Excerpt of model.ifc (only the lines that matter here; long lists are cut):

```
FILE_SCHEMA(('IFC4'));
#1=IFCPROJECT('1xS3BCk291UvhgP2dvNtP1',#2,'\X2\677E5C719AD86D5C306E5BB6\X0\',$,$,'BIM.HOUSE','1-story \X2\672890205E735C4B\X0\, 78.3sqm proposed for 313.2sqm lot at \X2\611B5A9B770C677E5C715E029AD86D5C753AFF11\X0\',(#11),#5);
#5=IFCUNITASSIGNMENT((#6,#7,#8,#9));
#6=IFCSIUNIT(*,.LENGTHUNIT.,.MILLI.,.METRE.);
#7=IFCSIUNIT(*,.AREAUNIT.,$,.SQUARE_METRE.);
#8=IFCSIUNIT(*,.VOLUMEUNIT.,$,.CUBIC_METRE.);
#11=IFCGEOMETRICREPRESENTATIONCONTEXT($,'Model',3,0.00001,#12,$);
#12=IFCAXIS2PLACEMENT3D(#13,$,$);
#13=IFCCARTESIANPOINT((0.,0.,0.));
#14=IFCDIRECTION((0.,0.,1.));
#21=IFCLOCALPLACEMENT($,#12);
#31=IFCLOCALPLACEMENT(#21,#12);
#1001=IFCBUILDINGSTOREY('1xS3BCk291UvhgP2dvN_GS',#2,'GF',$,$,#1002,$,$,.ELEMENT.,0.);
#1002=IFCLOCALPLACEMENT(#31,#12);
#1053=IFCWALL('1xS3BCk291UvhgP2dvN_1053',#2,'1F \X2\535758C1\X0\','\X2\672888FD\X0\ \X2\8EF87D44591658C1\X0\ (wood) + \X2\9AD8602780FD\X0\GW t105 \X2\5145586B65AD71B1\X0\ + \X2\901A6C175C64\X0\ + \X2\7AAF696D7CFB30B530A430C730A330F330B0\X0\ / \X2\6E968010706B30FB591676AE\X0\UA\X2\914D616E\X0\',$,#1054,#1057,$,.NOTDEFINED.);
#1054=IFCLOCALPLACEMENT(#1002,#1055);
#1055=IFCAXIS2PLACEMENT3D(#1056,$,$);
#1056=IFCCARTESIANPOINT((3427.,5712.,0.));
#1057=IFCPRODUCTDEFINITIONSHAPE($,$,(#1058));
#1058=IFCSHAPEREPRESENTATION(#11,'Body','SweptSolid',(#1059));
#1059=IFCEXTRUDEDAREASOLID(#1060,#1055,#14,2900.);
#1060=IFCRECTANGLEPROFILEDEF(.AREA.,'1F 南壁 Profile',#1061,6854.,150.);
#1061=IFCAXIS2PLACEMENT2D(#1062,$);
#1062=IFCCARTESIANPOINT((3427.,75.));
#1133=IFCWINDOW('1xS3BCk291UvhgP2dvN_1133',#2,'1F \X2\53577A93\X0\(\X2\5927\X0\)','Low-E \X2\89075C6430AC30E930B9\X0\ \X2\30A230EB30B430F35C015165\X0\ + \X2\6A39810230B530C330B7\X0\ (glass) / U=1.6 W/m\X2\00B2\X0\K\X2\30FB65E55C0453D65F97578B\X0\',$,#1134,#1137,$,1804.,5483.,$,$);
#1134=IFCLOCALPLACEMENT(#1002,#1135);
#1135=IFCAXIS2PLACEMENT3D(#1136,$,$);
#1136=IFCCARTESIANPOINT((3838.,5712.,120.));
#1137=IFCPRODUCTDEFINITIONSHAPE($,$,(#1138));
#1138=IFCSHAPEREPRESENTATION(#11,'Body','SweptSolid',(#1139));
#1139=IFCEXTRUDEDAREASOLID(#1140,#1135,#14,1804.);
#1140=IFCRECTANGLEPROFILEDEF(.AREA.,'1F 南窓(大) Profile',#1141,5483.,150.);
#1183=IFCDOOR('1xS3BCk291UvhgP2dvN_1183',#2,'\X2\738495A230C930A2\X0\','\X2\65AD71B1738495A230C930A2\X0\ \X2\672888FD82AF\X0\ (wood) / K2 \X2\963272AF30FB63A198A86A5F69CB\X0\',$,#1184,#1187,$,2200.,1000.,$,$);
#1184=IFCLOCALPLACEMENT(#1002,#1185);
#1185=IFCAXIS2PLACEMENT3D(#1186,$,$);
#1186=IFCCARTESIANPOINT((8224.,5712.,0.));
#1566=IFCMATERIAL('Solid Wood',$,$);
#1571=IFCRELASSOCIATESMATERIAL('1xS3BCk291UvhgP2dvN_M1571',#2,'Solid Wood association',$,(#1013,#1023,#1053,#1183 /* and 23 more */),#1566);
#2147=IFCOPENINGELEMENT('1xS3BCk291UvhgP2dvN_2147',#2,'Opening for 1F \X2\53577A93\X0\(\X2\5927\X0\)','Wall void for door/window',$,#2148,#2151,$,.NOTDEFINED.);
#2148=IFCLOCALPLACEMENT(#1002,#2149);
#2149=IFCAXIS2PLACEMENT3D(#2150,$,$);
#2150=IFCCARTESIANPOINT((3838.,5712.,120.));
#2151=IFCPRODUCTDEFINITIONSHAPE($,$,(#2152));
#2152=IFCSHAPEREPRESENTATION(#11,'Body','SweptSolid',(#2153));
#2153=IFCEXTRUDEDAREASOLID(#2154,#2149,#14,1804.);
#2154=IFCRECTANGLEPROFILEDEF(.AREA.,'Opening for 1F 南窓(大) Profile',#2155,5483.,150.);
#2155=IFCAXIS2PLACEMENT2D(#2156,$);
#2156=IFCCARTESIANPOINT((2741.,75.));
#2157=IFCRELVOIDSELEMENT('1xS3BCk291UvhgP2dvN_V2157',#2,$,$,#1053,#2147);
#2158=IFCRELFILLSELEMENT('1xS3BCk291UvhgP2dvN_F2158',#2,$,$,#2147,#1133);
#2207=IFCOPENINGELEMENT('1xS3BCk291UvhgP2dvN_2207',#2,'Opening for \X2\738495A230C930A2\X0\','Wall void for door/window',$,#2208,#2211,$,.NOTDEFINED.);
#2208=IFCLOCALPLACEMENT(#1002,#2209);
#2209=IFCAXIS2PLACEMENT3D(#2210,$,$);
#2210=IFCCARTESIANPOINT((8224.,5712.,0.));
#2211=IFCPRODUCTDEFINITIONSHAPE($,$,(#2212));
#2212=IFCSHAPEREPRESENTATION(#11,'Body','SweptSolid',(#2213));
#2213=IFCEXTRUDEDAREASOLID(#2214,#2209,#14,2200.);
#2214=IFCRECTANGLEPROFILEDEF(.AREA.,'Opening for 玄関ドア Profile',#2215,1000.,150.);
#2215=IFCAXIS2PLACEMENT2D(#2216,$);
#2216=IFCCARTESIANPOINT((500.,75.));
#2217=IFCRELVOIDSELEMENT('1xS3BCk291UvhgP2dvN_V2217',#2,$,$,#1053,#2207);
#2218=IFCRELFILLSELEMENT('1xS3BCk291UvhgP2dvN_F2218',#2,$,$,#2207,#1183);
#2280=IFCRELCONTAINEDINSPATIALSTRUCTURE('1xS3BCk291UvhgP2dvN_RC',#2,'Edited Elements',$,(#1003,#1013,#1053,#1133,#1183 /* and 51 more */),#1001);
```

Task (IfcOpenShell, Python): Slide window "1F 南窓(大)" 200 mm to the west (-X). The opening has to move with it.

```python
import ifcopenshell
import ifcopenshell.api.geometry
import ifcopenshell.util.placement
import ifcopenshell.util.unit

model = ifcopenshell.open("model.ifc")
unit_scale = ifcopenshell.util.unit.calculate_unit_scale(model)

window = model.by_id(1133)
opening = window.FillsVoids[0].RelatingOpeningElement
wall = opening.VoidsElements[0].RelatingBuildingElement

wall_matrix = ifcopenshell.util.placement.get_local_placement(wall.ObjectPlacement)
shift = wall_matrix[:3, 0] * -0.2 / unit_scale
before = ifcopenshell.util.placement.get_local_placement(window.ObjectPlacement)[:3, 3].copy()

# The window is not placed relative to its opening, so move both.
for product in (opening, window):
    matrix = ifcopenshell.util.placement.get_local_placement(product.ObjectPlacement)
    matrix[:3, 3] += shift
    ifcopenshell.api.geometry.edit_object_placement(model, product=product, matrix=matrix, is_si=False)

after = ifcopenshell.util.placement.get_local_placement(window.ObjectPlacement)[:3, 3]
print("window moved by", (after - before).round(3) + 0.0)

model.write("model_edited.ifc")
```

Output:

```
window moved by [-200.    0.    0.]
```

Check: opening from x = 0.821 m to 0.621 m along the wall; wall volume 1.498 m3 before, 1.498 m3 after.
